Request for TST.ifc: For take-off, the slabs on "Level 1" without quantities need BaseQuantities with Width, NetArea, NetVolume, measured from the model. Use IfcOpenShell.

First a look at what the model holds.

```python
import ifcopenshell
import ifcopenshell.util.element
import ifcopenshell.util.unit

model = ifcopenshell.open("TST.ifc")
print(model.schema)
for unit_type in ("LENGTHUNIT", "AREAUNIT", "VOLUMEUNIT"):
    print(unit_type, ifcopenshell.util.unit.calculate_unit_scale(model, unit_type))
storey = next(s for s in model.by_type("IfcBuildingStorey") if s.Name == "Level 1")
slabs = [e for e in ifcopenshell.util.element.get_decomposition(storey) if e.is_a("IfcSlab")]
for e in sorted(slabs, key=lambda e: e.id()):
    print(e.id(), e.is_a(), e.Name, list(ifcopenshell.util.element.get_psets(e, qtos_only=True)), sep=" | ")
```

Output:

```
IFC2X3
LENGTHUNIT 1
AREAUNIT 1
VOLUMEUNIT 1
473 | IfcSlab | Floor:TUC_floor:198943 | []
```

```python
import ifcopenshell
import ifcopenshell.api.pset
import ifcopenshell.geom
import ifcopenshell.util.element
import ifcopenshell.util.shape
import ifcopenshell.util.unit

model = ifcopenshell.open("TST.ifc")
unit_scale = ifcopenshell.util.unit.calculate_unit_scale(model)
area_scale = ifcopenshell.util.unit.calculate_unit_scale(model, "AREAUNIT")
volume_scale = ifcopenshell.util.unit.calculate_unit_scale(model, "VOLUMEUNIT")
settings = ifcopenshell.geom.settings()

storey = next(s for s in model.by_type("IfcBuildingStorey") if s.Name == "Level 1")
slabs = [e for e in ifcopenshell.util.element.get_decomposition(storey) if e.is_a("IfcSlab")]

for e in sorted(slabs, key=lambda e: e.id()):
    if ifcopenshell.util.element.get_psets(e, qtos_only=True, should_inherit=False):
        continue
    # Geometry comes back in metres, in the element's own axes.
    shape = ifcopenshell.geom.create_shape(settings, e)
    values = {
        "Width": ifcopenshell.util.shape.get_z(shape.geometry) / unit_scale,
        "NetArea": ifcopenshell.util.shape.get_footprint_area(shape.geometry) / area_scale,
        "NetVolume": ifcopenshell.util.shape.get_volume(shape.geometry) / volume_scale,
    }
    qto = ifcopenshell.api.pset.add_qto(model, product=e, name="BaseQuantities")
    ifcopenshell.api.pset.edit_qto(model, qto=qto, properties=values)
    print(e.id(), {k: round(v, 3) for k, v in values.items()})

model.write("TST_rev.ifc")
```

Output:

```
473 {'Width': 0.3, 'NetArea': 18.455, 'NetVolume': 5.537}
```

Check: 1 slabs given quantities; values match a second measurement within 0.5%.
